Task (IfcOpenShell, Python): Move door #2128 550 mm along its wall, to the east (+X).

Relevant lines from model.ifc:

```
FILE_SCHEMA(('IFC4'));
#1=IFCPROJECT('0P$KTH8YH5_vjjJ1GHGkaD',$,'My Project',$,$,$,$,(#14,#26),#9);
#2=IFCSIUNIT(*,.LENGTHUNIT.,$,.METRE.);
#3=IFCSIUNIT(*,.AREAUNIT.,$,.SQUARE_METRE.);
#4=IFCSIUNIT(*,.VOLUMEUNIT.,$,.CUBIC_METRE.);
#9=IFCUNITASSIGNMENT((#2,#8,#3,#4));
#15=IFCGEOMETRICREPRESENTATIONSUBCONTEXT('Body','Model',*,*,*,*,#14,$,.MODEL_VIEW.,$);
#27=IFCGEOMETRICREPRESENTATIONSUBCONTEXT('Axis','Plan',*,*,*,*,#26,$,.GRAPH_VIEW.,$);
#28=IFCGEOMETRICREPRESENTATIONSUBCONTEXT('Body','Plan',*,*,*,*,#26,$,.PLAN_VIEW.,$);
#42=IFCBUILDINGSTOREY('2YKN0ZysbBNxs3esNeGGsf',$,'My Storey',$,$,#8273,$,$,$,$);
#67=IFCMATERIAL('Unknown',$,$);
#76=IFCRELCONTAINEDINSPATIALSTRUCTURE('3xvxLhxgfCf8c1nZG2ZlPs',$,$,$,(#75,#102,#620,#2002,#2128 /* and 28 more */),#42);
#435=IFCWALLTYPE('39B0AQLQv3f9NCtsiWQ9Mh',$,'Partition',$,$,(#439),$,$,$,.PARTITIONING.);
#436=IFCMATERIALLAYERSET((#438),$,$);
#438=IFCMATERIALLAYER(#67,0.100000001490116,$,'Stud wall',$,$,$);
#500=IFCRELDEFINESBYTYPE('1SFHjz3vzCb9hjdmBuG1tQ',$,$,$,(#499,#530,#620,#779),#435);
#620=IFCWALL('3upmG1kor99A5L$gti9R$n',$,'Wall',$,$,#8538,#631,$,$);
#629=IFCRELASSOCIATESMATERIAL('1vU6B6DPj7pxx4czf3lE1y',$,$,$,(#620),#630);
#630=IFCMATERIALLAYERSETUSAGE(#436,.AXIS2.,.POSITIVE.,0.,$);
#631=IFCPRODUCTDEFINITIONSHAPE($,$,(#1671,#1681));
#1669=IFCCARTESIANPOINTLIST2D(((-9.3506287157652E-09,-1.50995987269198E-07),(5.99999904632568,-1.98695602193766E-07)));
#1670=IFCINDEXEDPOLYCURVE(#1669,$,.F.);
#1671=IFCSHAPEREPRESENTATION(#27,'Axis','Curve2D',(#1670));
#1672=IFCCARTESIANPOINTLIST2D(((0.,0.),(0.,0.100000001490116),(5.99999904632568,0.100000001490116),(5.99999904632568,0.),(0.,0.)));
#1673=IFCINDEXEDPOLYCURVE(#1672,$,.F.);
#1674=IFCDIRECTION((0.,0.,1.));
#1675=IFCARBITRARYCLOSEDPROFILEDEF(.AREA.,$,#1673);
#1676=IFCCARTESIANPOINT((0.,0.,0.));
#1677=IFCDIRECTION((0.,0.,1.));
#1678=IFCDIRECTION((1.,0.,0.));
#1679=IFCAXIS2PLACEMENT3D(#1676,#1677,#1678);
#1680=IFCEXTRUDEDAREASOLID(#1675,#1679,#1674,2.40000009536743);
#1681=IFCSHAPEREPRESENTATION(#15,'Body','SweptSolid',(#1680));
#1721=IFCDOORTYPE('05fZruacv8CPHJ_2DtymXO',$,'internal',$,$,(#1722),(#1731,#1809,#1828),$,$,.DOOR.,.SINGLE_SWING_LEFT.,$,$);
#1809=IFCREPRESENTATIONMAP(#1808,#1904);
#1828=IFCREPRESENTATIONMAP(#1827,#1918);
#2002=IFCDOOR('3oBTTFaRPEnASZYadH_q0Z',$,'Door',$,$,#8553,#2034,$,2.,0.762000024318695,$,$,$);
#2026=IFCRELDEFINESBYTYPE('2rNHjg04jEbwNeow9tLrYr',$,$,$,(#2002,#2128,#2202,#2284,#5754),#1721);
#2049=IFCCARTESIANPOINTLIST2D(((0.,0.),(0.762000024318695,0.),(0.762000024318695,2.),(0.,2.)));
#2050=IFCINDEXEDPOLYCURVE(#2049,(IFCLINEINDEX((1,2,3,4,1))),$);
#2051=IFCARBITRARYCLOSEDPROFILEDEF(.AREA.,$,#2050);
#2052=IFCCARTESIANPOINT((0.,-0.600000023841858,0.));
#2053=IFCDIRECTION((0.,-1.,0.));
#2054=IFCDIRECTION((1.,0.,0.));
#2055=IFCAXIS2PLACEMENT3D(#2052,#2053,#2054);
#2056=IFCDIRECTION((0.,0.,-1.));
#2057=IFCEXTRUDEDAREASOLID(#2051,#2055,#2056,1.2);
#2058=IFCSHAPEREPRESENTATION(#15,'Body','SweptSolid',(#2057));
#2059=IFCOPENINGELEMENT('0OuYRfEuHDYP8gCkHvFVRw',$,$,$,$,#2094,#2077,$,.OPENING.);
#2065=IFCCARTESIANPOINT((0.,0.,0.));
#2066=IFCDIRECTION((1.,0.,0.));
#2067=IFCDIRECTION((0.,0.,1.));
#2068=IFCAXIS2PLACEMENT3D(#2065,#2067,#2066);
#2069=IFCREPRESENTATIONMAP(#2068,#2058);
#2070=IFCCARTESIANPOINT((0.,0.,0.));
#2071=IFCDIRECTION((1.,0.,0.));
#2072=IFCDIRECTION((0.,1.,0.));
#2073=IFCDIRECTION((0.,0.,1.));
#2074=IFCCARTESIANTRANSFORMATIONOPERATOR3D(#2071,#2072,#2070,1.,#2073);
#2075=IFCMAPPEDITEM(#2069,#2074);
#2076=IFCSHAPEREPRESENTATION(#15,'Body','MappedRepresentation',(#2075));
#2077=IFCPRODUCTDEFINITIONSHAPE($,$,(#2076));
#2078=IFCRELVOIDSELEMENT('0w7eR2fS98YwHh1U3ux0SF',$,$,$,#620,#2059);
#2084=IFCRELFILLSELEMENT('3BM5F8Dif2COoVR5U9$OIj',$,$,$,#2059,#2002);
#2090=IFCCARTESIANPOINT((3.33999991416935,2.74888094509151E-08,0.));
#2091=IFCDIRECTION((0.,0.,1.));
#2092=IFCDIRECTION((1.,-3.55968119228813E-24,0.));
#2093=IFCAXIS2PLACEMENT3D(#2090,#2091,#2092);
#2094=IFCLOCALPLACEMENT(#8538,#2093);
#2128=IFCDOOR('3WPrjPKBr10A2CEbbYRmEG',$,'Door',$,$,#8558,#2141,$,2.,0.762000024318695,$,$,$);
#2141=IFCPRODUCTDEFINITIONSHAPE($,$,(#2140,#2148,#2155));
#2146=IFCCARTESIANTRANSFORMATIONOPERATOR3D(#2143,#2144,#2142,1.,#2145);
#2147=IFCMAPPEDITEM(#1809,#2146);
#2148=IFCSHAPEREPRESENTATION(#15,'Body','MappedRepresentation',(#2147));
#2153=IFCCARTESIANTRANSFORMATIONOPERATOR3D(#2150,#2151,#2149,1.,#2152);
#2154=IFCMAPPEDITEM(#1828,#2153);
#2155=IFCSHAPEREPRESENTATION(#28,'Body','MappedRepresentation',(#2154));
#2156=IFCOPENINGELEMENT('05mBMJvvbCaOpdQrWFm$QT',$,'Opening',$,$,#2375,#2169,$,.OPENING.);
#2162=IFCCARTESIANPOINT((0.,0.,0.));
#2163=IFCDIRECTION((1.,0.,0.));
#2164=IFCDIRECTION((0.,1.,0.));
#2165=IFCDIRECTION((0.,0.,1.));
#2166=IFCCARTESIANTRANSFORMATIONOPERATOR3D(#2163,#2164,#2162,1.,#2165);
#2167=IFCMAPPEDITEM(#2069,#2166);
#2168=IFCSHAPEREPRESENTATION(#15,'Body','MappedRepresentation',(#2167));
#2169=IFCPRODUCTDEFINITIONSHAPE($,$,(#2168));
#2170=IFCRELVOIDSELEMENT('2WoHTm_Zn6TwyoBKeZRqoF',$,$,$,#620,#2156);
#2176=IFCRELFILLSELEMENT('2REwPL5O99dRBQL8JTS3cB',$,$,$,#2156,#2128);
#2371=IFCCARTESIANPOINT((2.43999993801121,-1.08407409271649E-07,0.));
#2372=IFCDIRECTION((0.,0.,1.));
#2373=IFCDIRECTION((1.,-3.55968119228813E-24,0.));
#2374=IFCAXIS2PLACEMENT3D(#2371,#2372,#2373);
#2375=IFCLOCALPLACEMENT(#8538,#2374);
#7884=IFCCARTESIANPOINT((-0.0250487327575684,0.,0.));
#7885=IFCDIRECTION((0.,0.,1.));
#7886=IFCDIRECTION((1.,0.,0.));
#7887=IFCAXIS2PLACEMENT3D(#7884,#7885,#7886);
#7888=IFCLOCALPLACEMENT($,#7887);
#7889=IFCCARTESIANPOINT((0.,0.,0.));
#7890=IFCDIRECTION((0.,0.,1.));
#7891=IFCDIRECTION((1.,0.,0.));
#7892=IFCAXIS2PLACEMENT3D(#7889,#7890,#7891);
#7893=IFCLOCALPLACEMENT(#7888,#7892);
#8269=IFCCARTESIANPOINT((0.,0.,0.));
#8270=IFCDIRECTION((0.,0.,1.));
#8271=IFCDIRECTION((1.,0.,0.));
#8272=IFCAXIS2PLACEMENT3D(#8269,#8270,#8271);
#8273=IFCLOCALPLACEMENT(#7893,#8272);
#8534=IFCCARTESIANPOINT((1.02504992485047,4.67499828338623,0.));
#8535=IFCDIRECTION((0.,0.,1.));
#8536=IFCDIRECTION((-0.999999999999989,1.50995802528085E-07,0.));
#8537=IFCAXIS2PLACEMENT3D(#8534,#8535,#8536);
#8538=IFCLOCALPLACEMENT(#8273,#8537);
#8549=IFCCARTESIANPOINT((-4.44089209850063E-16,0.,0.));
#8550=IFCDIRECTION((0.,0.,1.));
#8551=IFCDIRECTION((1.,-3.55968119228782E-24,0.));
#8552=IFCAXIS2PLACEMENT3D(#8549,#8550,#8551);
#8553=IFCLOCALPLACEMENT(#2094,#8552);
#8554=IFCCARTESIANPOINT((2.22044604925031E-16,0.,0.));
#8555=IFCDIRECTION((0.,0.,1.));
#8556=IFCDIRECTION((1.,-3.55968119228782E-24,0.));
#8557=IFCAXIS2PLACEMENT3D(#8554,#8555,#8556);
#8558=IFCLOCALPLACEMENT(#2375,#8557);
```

```python
import ifcopenshell
import ifcopenshell.api.geometry
import ifcopenshell.util.placement

model = ifcopenshell.open("model.ifc")

door = model.by_guid("3WPrjPKBr10A2CEbbYRmEG")
opening = door.FillsVoids[0].RelatingOpeningElement
wall = opening.VoidsElements[0].RelatingBuildingElement

wall_matrix = ifcopenshell.util.placement.get_local_placement(wall.ObjectPlacement)
shift = wall_matrix[:3, 0] * -0.55
before = ifcopenshell.util.placement.get_local_placement(door.ObjectPlacement)[:3, 3].copy()

# The door is placed relative to its opening, so it follows when the opening moves.
matrix = ifcopenshell.util.placement.get_local_placement(opening.ObjectPlacement)
matrix[:3, 3] += shift
ifcopenshell.api.geometry.edit_object_placement(
    model, product=opening, matrix=matrix, is_si=False, should_transform_children=True
)

after = ifcopenshell.util.placement.get_local_placement(door.ObjectPlacement)[:3, 3]
print("door moved by", (after - before).round(3) + 0.0)

model.write("model_rev.ifc")
```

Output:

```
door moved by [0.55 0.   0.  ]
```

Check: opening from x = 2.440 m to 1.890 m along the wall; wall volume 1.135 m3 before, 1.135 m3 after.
